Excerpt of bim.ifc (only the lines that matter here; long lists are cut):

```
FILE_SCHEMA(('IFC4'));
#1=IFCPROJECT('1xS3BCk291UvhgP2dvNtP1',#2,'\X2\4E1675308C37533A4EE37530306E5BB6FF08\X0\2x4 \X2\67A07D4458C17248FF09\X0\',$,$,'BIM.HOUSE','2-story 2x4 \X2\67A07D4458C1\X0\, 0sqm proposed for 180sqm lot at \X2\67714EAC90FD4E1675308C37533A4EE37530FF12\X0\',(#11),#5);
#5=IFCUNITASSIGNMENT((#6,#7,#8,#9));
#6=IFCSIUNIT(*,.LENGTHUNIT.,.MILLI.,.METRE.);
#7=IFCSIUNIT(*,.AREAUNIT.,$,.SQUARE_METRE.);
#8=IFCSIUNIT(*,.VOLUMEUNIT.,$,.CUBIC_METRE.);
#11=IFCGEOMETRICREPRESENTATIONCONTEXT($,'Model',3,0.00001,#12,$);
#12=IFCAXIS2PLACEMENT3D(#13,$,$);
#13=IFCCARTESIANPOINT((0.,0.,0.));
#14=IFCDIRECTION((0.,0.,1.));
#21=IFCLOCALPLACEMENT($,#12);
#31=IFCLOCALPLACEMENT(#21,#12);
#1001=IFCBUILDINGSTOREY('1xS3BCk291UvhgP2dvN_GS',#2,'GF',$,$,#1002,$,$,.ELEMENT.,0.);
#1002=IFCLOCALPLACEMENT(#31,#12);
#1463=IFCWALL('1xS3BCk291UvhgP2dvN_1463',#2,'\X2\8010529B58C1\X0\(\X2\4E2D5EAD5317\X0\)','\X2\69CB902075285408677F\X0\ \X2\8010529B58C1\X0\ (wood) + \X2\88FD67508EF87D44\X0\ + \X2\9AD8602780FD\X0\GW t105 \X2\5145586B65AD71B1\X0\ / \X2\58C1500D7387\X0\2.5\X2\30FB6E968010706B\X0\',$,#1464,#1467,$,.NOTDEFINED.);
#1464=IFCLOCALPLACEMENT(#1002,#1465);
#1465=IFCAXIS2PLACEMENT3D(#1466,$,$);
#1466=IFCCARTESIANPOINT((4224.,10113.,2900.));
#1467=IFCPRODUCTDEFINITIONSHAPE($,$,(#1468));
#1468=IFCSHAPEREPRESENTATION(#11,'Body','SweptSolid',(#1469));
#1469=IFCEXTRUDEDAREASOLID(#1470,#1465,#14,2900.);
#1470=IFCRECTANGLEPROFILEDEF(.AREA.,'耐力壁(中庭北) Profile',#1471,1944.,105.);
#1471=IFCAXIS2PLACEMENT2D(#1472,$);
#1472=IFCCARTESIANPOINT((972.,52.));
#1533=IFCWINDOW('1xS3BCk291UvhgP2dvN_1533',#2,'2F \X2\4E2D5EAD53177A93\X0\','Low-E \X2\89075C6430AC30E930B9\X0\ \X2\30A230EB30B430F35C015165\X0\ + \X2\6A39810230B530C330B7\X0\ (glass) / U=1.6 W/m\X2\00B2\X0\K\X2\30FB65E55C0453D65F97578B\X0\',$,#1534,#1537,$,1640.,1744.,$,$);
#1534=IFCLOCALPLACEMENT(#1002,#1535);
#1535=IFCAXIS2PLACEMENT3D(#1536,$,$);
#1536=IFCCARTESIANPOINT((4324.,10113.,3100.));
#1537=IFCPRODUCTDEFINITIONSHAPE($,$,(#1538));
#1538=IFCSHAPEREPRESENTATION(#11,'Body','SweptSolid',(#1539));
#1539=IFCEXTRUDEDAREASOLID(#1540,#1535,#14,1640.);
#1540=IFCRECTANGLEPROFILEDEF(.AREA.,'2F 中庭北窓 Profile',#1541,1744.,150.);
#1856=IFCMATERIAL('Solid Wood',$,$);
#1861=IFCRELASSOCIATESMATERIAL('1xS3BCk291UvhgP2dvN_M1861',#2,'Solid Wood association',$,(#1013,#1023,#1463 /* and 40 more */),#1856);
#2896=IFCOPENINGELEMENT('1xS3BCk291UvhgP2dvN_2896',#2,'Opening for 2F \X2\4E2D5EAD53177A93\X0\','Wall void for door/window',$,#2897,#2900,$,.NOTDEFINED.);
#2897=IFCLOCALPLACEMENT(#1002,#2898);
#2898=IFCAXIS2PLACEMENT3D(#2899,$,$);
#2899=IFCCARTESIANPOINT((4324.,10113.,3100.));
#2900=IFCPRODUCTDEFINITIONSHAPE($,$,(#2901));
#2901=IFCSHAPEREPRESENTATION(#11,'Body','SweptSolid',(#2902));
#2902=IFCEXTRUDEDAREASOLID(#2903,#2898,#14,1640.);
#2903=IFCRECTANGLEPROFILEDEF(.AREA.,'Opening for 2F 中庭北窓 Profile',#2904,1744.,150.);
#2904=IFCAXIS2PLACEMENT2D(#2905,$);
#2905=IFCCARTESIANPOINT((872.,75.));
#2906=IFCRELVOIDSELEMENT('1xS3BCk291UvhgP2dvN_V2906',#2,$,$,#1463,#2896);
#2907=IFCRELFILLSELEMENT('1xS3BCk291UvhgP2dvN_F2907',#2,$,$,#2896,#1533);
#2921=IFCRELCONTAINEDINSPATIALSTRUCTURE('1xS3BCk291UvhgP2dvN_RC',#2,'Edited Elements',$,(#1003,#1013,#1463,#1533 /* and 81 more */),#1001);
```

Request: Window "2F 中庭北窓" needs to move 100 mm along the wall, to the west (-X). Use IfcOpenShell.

```python
import ifcopenshell
import ifcopenshell.api.geometry
import ifcopenshell.util.placement

model = ifcopenshell.open("bim.ifc")

window = model.by_guid("1xS3BCk291UvhgP2dvN_1533")
opening = window.FillsVoids[0].RelatingOpeningElement
wall = opening.VoidsElements[0].RelatingBuildingElement

wall_matrix = ifcopenshell.util.placement.get_local_placement(wall.ObjectPlacement)
shift = wall_matrix[:3, 0] * -100.0
before = ifcopenshell.util.placement.get_local_placement(window.ObjectPlacement)[:3, 3].copy()

# The window is not placed relative to its opening, so move both.
for product in (opening, window):
    matrix = ifcopenshell.util.placement.get_local_placement(product.ObjectPlacement)
    matrix[:3, 3] += shift
    ifcopenshell.api.geometry.edit_object_placement(model, product=product, matrix=matrix, is_si=False)

after = ifcopenshell.util.placement.get_local_placement(window.ObjectPlacement)[:3, 3]
print("window moved by", (after - before).round(3) + 0.0)

model.write("bim_rev.ifc")
```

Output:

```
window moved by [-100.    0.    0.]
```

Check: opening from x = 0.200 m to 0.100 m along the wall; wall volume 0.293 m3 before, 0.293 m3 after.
